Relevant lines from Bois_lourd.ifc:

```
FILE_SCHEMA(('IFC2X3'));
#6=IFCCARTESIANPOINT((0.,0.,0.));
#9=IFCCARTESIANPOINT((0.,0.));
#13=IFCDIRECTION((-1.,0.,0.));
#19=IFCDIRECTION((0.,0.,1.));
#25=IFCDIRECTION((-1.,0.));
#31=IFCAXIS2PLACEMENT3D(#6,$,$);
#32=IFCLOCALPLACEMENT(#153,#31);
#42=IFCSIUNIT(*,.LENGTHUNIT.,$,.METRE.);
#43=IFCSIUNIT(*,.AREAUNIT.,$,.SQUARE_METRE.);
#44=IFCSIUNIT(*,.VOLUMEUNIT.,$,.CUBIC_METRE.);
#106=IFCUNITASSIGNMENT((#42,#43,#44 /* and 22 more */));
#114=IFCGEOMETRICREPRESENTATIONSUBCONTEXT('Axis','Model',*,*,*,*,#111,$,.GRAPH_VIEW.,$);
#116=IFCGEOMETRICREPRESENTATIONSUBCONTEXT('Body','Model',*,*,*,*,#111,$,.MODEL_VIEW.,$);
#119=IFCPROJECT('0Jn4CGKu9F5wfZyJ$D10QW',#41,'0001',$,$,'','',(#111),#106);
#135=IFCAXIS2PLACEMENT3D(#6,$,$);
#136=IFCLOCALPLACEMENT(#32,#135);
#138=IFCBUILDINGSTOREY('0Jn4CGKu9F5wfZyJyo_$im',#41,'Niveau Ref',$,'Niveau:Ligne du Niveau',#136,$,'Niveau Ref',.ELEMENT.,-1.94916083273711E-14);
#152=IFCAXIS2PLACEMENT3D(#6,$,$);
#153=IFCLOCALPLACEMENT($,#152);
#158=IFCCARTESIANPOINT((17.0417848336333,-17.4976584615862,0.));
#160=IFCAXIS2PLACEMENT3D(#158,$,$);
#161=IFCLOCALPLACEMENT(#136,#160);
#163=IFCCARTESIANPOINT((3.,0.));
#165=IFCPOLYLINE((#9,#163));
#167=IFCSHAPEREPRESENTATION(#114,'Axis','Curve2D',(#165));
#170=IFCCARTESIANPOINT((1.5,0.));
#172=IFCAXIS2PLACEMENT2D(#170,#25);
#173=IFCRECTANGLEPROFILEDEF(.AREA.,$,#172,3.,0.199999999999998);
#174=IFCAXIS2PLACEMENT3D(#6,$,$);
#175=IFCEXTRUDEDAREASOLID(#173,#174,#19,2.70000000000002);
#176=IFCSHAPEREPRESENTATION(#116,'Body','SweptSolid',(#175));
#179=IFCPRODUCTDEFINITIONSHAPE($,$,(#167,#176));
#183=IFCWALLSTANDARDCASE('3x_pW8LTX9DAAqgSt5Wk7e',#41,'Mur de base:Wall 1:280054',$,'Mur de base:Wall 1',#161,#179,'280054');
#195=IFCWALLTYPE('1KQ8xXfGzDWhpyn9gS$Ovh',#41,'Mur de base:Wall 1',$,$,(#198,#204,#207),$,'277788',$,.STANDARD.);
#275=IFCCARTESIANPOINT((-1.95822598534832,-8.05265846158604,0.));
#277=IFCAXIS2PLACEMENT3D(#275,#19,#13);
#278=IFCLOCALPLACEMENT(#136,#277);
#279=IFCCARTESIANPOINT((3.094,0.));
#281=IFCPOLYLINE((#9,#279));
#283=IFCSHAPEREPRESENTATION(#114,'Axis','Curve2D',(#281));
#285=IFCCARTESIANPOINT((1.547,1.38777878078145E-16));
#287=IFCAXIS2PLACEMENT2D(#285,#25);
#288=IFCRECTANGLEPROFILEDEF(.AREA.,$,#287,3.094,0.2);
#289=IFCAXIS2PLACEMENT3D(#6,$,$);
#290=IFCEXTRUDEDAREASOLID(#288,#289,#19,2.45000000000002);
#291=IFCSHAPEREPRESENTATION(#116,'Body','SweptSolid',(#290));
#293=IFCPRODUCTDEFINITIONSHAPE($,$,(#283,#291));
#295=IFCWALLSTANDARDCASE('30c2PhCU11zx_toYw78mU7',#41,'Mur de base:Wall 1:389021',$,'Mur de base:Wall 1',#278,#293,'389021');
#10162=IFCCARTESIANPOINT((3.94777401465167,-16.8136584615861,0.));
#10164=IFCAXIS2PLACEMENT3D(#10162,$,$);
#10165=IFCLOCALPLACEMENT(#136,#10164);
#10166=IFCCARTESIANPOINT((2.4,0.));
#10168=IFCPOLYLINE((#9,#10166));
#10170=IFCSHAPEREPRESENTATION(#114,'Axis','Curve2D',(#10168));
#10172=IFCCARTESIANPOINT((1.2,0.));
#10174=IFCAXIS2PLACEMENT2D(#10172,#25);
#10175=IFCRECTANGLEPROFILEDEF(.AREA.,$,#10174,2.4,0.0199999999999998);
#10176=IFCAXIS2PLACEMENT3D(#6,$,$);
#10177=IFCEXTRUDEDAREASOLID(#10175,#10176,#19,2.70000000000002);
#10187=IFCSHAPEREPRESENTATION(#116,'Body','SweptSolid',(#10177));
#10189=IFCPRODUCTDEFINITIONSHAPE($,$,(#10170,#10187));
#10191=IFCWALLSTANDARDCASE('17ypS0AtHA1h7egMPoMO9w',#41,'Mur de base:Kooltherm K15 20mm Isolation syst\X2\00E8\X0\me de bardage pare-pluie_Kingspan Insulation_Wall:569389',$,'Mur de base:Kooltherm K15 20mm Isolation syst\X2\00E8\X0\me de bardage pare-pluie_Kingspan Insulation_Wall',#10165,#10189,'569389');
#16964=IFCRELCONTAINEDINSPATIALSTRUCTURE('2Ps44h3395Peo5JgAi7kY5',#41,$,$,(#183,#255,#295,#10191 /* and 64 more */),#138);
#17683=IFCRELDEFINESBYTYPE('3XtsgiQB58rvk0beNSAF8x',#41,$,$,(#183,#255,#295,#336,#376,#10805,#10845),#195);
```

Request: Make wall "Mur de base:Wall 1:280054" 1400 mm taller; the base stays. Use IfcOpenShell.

```python
import ifcopenshell
import ifcopenshell.geom
import ifcopenshell.util.representation
import ifcopenshell.util.shape
import ifcopenshell.util.unit

model = ifcopenshell.open("Bois_lourd.ifc")
unit_scale = ifcopenshell.util.unit.calculate_unit_scale(model)
settings = ifcopenshell.geom.settings()


def volume(element):
    """Net volume in cubic metres, openings subtracted."""
    shape = ifcopenshell.geom.create_shape(settings, element)
    return ifcopenshell.util.shape.get_volume(shape.geometry)


wall = model.by_guid("3x_pW8LTX9DAAqgSt5Wk7e")
before = volume(wall)

body = ifcopenshell.util.representation.get_representation(wall, "Model", "Body")
solid = body.Items[0]
old_height = solid.Depth
solid.Depth += 1.4 / unit_scale
after = volume(wall)

print(f"height {old_height:g} -> {solid.Depth:g}, volume {before:.3f} -> {after:.3f} m3")

model.write("Bois_lourd_rev.ifc")
```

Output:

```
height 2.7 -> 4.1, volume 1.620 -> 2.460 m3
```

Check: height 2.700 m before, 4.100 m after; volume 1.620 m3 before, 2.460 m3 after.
